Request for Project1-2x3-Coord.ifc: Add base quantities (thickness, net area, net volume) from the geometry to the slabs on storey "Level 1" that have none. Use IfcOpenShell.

First a look at what the model holds.

```python
import ifcopenshell
import ifcopenshell.util.element
import ifcopenshell.util.unit

model = ifcopenshell.open("Project1-2x3-Coord.ifc")
print(model.schema)
for unit_type in ("LENGTHUNIT", "AREAUNIT", "VOLUMEUNIT"):
    print(unit_type, ifcopenshell.util.unit.calculate_unit_scale(model, unit_type))
storey = next(s for s in model.by_type("IfcBuildingStorey") if s.Name == "Level 1")
slabs = [e for e in ifcopenshell.util.element.get_decomposition(storey) if e.is_a("IfcSlab")]
for e in sorted(slabs, key=lambda e: e.id()):
    print(e.id(), e.is_a(), e.Name, list(ifcopenshell.util.element.get_psets(e, qtos_only=True)), sep=" | ")
```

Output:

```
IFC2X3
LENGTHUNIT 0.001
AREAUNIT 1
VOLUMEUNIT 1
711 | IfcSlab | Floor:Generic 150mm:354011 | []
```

```python
import ifcopenshell
import ifcopenshell.api.pset
import ifcopenshell.geom
import ifcopenshell.util.element
import ifcopenshell.util.shape
import ifcopenshell.util.unit

model = ifcopenshell.open("Project1-2x3-Coord.ifc")
unit_scale = ifcopenshell.util.unit.calculate_unit_scale(model)
area_scale = ifcopenshell.util.unit.calculate_unit_scale(model, "AREAUNIT")
volume_scale = ifcopenshell.util.unit.calculate_unit_scale(model, "VOLUMEUNIT")
settings = ifcopenshell.geom.settings()

storey = next(s for s in model.by_type("IfcBuildingStorey") if s.Name == "Level 1")
slabs = [e for e in ifcopenshell.util.element.get_decomposition(storey) if e.is_a("IfcSlab")]

for e in sorted(slabs, key=lambda e: e.id()):
    if ifcopenshell.util.element.get_psets(e, qtos_only=True, should_inherit=False):
        continue
    # Geometry comes back in metres, in the element's own axes.
    shape = ifcopenshell.geom.create_shape(settings, e)
    values = {
        "Width": ifcopenshell.util.shape.get_z(shape.geometry) / unit_scale,
        "NetArea": ifcopenshell.util.shape.get_footprint_area(shape.geometry) / area_scale,
        "NetVolume": ifcopenshell.util.shape.get_volume(shape.geometry) / volume_scale,
    }
    qto = ifcopenshell.api.pset.add_qto(model, product=e, name="BaseQuantities")
    ifcopenshell.api.pset.edit_qto(model, qto=qto, properties=values)
    print(e.id(), {k: round(v, 3) for k, v in values.items()})

model.write("Project1-2x3-Coord_edited.ifc")
```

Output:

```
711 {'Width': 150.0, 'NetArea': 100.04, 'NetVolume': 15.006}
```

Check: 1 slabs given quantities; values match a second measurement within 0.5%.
